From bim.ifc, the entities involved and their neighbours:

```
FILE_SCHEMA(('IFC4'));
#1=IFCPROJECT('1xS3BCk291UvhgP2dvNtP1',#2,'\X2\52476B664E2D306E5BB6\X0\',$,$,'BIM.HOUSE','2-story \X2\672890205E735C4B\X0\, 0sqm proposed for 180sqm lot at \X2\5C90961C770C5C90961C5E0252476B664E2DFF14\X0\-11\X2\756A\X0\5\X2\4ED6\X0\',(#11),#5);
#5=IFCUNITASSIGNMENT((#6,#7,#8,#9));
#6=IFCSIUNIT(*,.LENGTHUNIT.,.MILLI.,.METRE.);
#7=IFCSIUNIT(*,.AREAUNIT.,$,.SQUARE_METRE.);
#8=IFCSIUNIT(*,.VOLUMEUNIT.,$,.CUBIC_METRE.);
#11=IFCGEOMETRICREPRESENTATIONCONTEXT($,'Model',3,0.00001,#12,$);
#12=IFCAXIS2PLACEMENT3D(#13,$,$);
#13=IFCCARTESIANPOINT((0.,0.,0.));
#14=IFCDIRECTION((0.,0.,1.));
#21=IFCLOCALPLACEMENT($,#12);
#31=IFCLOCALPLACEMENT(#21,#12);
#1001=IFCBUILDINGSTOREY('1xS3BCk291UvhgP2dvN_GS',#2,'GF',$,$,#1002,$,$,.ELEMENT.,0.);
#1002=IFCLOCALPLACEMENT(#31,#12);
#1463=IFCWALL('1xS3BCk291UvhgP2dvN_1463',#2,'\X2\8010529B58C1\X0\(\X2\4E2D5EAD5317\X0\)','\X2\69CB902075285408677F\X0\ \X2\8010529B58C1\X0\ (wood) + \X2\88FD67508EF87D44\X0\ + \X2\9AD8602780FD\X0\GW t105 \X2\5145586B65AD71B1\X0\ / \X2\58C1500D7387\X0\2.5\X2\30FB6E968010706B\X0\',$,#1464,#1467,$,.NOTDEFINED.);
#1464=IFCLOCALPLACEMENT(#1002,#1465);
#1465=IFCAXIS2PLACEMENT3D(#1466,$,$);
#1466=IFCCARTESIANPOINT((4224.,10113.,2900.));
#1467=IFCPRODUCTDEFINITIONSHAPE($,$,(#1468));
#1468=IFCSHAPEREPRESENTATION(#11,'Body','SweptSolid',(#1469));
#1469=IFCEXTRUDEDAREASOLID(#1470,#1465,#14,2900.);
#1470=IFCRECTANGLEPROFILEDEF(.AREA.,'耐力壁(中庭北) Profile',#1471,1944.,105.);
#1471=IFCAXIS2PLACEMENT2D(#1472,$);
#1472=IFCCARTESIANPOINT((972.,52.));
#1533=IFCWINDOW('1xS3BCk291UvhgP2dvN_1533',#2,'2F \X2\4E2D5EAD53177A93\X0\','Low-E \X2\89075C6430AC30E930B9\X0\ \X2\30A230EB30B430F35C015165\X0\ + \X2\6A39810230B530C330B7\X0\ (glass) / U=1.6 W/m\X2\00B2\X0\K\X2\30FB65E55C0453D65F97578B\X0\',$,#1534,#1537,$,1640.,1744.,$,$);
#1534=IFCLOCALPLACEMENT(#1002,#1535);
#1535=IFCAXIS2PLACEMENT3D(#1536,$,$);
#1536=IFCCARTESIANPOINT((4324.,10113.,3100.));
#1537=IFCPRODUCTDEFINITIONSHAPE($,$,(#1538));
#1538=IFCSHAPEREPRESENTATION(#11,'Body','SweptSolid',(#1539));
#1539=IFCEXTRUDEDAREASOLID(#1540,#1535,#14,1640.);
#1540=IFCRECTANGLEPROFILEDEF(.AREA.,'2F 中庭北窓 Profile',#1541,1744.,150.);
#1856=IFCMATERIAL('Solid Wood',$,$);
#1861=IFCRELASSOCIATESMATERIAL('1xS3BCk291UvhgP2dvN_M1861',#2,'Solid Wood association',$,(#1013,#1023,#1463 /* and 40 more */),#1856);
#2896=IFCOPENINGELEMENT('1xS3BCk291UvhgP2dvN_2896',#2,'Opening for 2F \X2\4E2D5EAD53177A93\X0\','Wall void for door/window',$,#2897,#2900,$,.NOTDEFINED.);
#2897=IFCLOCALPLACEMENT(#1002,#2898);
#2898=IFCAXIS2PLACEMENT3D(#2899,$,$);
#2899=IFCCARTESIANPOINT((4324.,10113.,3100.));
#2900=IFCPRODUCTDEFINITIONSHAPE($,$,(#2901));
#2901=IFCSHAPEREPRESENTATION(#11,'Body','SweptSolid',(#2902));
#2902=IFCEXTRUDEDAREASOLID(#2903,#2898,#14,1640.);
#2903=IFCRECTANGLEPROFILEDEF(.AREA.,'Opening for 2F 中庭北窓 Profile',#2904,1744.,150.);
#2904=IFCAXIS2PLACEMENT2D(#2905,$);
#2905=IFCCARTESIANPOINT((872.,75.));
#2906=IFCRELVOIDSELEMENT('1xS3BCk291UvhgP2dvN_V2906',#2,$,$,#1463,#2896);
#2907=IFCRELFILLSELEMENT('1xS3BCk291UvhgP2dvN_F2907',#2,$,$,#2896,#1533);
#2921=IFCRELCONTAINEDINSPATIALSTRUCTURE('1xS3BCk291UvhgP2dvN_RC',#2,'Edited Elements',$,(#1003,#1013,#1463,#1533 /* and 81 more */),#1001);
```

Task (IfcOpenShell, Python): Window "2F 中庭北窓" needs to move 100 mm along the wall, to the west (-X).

```python
import ifcopenshell
import ifcopenshell.api.geometry
import ifcopenshell.util.placement
import ifcopenshell.util.unit

model = ifcopenshell.open("bim.ifc")
unit_scale = ifcopenshell.util.unit.calculate_unit_scale(model)

window = model.by_id(1533)
opening = window.FillsVoids[0].RelatingOpeningElement
wall = opening.VoidsElements[0].RelatingBuildingElement

wall_matrix = ifcopenshell.util.placement.get_local_placement(wall.ObjectPlacement)
shift = wall_matrix[:3, 0] * -0.1 / unit_scale
before = ifcopenshell.util.placement.get_local_placement(window.ObjectPlacement)[:3, 3].copy()

# The window is not placed relative to its opening, so move both.
for product in (opening, window):
    matrix = ifcopenshell.util.placement.get_local_placement(product.ObjectPlacement)
    matrix[:3, 3] += shift
    ifcopenshell.api.geometry.edit_object_placement(model, product=product, matrix=matrix, is_si=False)

after = ifcopenshell.util.placement.get_local_placement(window.ObjectPlacement)[:3, 3]
print("window moved by", (after - before).round(3) + 0.0)

model.write("bim_v2.ifc")
```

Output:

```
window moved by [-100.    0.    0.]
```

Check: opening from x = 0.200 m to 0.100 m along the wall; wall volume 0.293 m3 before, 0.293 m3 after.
